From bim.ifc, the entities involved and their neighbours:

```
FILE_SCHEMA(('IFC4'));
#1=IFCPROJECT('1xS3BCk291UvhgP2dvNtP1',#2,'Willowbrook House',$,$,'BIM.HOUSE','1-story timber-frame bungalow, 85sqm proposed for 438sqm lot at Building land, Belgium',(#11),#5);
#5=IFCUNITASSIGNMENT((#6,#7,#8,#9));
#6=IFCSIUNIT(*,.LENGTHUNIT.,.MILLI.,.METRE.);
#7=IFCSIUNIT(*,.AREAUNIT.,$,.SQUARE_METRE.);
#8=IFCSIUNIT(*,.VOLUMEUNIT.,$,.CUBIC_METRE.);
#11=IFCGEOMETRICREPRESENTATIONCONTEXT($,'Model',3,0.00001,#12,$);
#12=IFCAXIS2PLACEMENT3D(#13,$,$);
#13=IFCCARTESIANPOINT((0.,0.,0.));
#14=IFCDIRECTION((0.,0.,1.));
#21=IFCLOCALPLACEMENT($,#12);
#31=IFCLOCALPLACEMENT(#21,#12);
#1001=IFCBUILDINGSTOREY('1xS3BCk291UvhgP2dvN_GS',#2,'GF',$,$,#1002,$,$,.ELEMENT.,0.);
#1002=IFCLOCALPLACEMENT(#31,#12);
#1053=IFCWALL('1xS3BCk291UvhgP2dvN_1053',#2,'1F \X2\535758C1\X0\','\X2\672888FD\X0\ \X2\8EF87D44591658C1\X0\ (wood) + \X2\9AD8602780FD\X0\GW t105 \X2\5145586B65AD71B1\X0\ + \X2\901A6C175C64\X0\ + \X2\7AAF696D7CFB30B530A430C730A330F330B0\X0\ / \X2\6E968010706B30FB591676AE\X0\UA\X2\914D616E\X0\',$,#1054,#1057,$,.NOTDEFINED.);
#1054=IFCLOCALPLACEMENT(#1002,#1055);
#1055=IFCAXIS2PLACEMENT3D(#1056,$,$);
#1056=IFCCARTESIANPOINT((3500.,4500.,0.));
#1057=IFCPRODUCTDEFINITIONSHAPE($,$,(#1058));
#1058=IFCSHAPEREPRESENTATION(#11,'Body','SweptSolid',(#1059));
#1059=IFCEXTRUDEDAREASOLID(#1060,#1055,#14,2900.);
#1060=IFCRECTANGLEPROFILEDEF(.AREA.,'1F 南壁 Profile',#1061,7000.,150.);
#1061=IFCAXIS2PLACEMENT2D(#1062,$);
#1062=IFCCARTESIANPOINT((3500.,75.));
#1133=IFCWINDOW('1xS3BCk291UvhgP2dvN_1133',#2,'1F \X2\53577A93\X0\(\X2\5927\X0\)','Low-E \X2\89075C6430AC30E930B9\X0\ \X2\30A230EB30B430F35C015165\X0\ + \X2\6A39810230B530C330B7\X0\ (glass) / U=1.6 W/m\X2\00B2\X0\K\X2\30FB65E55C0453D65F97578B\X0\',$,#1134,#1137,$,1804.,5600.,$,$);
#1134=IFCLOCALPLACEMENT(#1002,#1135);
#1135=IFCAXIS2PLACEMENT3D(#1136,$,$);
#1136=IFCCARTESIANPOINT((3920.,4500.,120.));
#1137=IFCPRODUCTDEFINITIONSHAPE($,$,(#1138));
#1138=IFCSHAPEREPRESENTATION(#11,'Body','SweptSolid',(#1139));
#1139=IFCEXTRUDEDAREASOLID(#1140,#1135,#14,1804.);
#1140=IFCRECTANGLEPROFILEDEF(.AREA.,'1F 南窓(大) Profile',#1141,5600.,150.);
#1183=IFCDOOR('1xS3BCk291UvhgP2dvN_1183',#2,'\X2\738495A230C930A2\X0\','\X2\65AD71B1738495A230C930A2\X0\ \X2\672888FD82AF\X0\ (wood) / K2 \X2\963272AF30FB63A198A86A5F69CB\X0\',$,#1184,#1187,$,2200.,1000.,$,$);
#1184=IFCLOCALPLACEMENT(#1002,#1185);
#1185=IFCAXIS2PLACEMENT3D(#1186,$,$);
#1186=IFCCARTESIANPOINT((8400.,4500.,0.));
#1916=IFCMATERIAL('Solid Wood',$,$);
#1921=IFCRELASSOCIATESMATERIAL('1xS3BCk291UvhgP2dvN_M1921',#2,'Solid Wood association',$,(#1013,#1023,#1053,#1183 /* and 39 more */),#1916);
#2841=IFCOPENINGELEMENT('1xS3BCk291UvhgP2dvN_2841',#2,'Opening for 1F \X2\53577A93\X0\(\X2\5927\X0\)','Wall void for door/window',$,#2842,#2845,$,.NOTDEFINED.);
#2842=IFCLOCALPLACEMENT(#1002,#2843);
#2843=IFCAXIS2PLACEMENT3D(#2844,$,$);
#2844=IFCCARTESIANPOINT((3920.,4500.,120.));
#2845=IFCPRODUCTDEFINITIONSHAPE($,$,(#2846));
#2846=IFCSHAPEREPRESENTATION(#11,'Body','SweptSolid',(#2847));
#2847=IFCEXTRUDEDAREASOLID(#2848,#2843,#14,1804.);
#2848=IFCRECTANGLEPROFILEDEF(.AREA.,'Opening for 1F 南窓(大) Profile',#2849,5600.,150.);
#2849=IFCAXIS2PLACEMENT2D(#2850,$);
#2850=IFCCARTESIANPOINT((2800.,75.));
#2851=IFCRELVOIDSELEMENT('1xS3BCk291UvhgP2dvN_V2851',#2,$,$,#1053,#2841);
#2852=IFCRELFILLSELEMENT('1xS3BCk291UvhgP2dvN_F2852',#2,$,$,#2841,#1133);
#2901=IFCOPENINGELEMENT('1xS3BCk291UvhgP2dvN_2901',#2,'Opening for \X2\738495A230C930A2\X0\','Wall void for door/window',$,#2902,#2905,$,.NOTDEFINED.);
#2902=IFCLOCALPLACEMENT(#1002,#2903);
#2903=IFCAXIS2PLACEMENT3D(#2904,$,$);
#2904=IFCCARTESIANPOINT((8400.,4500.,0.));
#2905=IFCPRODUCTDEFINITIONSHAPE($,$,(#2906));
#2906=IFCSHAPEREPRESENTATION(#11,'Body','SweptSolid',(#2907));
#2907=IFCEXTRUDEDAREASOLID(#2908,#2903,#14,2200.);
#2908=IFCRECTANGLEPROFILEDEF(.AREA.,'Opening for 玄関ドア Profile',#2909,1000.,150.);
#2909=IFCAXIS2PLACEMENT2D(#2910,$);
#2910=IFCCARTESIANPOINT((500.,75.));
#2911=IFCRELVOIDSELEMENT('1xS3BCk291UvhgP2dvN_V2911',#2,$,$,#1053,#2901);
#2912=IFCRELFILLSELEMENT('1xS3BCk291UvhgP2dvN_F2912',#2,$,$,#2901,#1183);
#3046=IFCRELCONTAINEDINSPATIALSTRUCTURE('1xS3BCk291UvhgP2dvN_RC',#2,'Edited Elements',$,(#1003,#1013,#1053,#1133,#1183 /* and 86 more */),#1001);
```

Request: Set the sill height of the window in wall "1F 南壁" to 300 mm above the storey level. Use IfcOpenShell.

```python
import numpy as np
import ifcopenshell
import ifcopenshell.api.geometry
import ifcopenshell.geom
import ifcopenshell.util.element
import ifcopenshell.util.placement
import ifcopenshell.util.shape
import ifcopenshell.util.unit

model = ifcopenshell.open("bim.ifc")
unit_scale = ifcopenshell.util.unit.calculate_unit_scale(model)

window = model.by_guid("1xS3BCk291UvhgP2dvN_1133")
opening = window.FillsVoids[0].RelatingOpeningElement
storey = ifcopenshell.util.element.get_container(window, ifc_class="IfcBuildingStorey")
level = ifcopenshell.util.placement.get_local_placement(storey.ObjectPlacement)[2, 3]

# The opening's origin need not be at the sill, so measure its lowest point.
shape = ifcopenshell.geom.create_shape(ifcopenshell.geom.settings(), opening)
bottom = ifcopenshell.util.shape.get_shape_bottom_elevation(shape, shape.geometry) / unit_scale
dz = level + 0.3 / unit_scale - bottom

shift = np.array([0.0, 0.0, dz])
# The window is not placed relative to its opening, so move both.
for product in (opening, window):
    matrix = ifcopenshell.util.placement.get_local_placement(product.ObjectPlacement)
    matrix[:3, 3] += shift
    ifcopenshell.api.geometry.edit_object_placement(model, product=product, matrix=matrix, is_si=False)

print(f"moved by {dz * unit_scale:+.3f} m")

model.write("bim_v2.ifc")
```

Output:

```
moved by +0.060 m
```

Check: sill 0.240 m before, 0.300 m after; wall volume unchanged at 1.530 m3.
